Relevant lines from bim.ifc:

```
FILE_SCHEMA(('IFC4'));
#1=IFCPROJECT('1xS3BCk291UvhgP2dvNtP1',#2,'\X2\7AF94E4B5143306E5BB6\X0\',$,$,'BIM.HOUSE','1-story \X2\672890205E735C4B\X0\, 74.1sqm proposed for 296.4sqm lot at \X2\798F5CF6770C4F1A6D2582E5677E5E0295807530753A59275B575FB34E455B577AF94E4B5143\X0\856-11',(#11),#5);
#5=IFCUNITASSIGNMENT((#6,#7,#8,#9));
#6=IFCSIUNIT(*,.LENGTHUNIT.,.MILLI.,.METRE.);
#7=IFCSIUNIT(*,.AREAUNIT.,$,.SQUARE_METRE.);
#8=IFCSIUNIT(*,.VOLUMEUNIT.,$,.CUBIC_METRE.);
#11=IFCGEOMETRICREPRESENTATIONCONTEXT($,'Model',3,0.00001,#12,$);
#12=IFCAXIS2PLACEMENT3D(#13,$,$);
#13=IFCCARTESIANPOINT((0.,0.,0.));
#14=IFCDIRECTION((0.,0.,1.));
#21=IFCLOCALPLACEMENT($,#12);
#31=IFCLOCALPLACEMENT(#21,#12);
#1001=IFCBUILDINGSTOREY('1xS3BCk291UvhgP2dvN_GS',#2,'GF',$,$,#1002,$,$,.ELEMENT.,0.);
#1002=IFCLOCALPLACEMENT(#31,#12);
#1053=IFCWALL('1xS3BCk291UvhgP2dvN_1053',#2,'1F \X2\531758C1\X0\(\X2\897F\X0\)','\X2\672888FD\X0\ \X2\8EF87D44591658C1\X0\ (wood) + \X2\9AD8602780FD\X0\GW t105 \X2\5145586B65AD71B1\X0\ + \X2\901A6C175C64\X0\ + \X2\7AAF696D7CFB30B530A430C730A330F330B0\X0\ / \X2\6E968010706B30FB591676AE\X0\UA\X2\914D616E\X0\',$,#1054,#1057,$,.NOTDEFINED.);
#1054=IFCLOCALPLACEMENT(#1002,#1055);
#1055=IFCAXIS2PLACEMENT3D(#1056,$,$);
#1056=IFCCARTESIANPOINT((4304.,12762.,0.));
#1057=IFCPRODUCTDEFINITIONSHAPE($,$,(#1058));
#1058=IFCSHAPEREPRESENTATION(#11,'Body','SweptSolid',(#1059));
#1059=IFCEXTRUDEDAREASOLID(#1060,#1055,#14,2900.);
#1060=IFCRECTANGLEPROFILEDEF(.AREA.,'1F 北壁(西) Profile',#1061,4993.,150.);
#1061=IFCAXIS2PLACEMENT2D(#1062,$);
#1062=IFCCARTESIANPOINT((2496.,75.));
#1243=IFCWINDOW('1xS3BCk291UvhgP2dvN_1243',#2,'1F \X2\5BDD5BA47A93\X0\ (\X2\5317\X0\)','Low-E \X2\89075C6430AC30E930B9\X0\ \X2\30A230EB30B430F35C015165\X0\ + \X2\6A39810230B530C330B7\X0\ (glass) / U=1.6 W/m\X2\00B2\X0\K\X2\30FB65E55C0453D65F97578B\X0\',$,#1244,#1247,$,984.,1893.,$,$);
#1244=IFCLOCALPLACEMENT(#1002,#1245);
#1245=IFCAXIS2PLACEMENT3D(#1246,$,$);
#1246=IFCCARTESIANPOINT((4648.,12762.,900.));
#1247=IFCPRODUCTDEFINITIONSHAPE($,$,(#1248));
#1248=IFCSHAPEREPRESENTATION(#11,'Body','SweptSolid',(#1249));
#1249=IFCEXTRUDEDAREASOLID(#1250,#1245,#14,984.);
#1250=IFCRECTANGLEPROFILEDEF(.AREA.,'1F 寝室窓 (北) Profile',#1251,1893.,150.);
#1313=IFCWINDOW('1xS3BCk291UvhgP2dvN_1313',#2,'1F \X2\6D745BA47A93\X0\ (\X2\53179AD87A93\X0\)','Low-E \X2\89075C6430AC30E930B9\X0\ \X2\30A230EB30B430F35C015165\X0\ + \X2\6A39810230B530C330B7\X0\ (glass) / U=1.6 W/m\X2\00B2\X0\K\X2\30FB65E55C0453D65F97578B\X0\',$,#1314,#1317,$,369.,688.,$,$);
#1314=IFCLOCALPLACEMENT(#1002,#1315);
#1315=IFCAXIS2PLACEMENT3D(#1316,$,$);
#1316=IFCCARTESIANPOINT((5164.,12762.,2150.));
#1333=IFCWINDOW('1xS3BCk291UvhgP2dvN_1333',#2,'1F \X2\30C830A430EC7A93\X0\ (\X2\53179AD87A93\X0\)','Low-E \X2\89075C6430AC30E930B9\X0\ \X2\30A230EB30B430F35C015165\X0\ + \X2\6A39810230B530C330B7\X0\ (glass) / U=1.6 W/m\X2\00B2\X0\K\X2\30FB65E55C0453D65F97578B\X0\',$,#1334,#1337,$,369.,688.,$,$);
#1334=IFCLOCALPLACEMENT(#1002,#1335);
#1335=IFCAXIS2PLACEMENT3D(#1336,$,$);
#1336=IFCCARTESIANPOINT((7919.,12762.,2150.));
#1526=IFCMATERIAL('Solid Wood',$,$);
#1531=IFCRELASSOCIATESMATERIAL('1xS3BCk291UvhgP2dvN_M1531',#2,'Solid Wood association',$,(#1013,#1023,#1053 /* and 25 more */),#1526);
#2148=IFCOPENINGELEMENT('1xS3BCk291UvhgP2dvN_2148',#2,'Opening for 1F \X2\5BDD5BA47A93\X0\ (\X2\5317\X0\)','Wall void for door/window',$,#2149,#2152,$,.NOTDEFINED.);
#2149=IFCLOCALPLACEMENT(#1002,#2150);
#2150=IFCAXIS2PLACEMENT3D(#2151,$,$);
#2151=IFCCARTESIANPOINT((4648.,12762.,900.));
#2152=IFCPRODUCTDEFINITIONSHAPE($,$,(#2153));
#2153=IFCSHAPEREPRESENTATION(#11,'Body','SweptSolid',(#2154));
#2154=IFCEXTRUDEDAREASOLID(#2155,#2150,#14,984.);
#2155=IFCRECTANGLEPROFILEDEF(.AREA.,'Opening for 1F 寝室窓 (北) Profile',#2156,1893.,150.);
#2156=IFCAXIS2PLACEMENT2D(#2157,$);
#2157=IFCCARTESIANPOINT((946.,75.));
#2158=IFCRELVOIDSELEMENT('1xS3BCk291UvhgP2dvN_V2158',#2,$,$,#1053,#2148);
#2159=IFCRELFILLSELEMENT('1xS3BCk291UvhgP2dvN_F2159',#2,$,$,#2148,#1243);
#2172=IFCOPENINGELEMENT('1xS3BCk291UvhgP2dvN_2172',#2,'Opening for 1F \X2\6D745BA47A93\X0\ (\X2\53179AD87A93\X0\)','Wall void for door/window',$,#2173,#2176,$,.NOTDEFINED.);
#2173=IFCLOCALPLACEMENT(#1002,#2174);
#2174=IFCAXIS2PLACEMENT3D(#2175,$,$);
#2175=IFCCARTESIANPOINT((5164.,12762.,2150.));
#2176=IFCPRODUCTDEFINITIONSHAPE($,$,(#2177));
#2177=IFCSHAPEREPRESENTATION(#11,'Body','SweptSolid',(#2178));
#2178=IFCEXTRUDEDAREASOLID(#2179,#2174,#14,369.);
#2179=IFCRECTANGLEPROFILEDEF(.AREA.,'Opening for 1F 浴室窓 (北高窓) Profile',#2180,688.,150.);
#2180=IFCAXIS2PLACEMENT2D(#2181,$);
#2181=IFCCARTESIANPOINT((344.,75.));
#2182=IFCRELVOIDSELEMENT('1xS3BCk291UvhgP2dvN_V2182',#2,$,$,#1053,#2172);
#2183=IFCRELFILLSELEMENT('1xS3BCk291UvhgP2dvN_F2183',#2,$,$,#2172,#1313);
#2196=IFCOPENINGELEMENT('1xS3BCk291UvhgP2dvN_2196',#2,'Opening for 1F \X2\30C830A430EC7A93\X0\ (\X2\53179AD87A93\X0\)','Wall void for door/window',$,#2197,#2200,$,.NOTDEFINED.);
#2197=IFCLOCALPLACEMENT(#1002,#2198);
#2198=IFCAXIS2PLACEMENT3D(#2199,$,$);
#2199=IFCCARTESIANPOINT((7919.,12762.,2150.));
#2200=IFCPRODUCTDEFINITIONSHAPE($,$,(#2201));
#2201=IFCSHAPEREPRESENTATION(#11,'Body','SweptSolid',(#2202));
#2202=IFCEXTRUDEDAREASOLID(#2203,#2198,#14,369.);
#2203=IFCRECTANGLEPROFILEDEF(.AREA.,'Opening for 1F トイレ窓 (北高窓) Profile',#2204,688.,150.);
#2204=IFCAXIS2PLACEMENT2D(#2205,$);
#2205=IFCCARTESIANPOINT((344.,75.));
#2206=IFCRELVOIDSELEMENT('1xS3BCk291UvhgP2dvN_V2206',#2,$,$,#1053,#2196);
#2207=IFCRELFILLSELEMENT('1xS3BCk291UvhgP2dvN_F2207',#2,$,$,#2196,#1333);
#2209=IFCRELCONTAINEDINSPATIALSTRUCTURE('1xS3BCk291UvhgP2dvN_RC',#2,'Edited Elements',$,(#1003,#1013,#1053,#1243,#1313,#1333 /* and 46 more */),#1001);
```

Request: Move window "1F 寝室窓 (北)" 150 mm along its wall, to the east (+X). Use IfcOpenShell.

```python
import ifcopenshell
import ifcopenshell.api.geometry
import ifcopenshell.util.placement

model = ifcopenshell.open("bim.ifc")

window = model.by_guid("1xS3BCk291UvhgP2dvN_1243")
opening = window.FillsVoids[0].RelatingOpeningElement
wall = opening.VoidsElements[0].RelatingBuildingElement

wall_matrix = ifcopenshell.util.placement.get_local_placement(wall.ObjectPlacement)
shift = wall_matrix[:3, 0] * 150.0
before = ifcopenshell.util.placement.get_local_placement(window.ObjectPlacement)[:3, 3].copy()

# The window is not placed relative to its opening, so move both.
for product in (opening, window):
    matrix = ifcopenshell.util.placement.get_local_placement(product.ObjectPlacement)
    matrix[:3, 3] += shift
    ifcopenshell.api.geometry.edit_object_placement(model, product=product, matrix=matrix, is_si=False)

after = ifcopenshell.util.placement.get_local_placement(window.ObjectPlacement)[:3, 3]
print("window moved by", (after - before).round(3) + 0.0)

model.write("bim_v2.ifc")
```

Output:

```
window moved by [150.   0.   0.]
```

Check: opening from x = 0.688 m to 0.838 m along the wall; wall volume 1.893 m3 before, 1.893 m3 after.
